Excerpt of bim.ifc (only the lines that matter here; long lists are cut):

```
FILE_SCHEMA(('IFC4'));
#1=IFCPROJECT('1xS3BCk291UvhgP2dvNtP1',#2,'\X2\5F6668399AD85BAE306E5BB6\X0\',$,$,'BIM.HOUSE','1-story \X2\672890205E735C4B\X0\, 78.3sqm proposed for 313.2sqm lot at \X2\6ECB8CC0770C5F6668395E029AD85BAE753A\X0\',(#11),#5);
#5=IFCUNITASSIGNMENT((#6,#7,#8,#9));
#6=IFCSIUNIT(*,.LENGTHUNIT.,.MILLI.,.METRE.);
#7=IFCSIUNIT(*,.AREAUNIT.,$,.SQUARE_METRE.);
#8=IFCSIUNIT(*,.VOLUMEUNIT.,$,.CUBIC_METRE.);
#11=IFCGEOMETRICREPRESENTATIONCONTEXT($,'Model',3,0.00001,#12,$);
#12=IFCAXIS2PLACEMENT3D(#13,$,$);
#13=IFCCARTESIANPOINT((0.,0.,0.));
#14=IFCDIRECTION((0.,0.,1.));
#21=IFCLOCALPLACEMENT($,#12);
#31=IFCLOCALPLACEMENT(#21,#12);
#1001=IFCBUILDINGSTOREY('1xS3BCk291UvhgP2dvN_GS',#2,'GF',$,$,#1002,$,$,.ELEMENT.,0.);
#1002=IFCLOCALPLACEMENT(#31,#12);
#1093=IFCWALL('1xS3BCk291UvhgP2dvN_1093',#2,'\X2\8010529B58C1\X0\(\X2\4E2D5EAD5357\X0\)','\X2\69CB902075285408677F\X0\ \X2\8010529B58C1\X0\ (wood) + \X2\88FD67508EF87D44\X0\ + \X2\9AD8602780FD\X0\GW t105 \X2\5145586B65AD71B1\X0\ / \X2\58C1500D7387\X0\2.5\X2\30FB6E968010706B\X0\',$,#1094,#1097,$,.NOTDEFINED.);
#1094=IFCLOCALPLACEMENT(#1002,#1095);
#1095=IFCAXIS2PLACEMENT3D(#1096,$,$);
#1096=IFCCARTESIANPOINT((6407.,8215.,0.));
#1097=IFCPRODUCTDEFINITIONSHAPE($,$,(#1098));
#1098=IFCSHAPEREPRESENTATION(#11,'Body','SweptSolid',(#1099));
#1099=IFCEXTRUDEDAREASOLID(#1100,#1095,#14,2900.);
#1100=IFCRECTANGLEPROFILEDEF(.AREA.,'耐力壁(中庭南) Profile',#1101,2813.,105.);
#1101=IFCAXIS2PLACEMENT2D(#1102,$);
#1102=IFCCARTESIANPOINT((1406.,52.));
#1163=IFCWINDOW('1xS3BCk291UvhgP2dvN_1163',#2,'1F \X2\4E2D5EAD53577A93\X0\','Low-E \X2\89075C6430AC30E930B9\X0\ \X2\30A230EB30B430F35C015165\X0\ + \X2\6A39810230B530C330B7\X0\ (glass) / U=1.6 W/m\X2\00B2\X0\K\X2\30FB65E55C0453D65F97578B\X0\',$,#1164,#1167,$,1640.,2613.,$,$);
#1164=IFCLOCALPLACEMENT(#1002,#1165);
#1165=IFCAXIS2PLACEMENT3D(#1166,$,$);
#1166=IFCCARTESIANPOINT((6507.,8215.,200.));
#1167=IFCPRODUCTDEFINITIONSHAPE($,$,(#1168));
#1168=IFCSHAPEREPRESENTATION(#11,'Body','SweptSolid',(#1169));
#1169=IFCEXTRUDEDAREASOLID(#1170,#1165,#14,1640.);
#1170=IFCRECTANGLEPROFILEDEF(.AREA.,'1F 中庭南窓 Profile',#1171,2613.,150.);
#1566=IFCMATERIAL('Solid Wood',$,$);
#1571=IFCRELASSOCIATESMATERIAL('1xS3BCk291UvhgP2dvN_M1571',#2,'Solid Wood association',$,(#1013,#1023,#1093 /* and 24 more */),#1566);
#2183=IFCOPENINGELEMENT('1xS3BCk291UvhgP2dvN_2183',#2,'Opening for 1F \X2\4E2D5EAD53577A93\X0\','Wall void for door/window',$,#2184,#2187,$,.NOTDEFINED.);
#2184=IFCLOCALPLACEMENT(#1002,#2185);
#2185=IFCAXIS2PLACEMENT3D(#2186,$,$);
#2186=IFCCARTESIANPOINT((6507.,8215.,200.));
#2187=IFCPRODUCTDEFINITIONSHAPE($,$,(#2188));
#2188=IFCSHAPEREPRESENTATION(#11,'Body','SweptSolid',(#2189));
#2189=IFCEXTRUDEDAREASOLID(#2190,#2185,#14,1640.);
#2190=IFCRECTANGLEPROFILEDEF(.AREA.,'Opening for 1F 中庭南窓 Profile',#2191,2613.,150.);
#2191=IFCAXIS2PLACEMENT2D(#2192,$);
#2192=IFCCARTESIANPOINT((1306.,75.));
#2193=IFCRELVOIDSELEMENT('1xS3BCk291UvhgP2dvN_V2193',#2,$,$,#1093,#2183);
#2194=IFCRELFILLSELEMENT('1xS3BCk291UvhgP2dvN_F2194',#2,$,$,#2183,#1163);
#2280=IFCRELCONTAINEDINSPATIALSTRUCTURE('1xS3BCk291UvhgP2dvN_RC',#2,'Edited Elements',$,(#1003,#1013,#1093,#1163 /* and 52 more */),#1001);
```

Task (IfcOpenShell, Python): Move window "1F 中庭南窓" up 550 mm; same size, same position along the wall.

```python
import numpy as np
import ifcopenshell
import ifcopenshell.api.geometry
import ifcopenshell.util.placement
import ifcopenshell.util.unit

model = ifcopenshell.open("bim.ifc")
unit_scale = ifcopenshell.util.unit.calculate_unit_scale(model)

window = model.by_guid("1xS3BCk291UvhgP2dvN_1163")
opening = window.FillsVoids[0].RelatingOpeningElement
dz = 0.55 / unit_scale

shift = np.array([0.0, 0.0, dz])
# The window is not placed relative to its opening, so move both.
for product in (opening, window):
    matrix = ifcopenshell.util.placement.get_local_placement(product.ObjectPlacement)
    matrix[:3, 3] += shift
    ifcopenshell.api.geometry.edit_object_placement(model, product=product, matrix=matrix, is_si=False)

print(f"moved by {dz * unit_scale:+.3f} m")

model.write("bim-out.ifc")
```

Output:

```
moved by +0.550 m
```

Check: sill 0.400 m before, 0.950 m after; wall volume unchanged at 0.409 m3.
